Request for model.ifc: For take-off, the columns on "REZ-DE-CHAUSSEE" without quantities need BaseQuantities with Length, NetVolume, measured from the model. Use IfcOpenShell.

First a look at what the model holds.

```python
import ifcopenshell
import ifcopenshell.util.element
import ifcopenshell.util.unit

model = ifcopenshell.open("model.ifc")
print(model.schema)
for unit_type in ("LENGTHUNIT", "AREAUNIT", "VOLUMEUNIT"):
    print(unit_type, ifcopenshell.util.unit.calculate_unit_scale(model, unit_type))
storey = next(s for s in model.by_type("IfcBuildingStorey") if s.Name == "REZ-DE-CHAUSSEE")
columns = [e for e in ifcopenshell.util.element.get_decomposition(storey) if e.is_a("IfcColumn")]
for e in sorted(columns, key=lambda e: e.id()):
    print(e.id(), e.is_a(), e.Name, list(ifcopenshell.util.element.get_psets(e, qtos_only=True)), sep=" | ")
```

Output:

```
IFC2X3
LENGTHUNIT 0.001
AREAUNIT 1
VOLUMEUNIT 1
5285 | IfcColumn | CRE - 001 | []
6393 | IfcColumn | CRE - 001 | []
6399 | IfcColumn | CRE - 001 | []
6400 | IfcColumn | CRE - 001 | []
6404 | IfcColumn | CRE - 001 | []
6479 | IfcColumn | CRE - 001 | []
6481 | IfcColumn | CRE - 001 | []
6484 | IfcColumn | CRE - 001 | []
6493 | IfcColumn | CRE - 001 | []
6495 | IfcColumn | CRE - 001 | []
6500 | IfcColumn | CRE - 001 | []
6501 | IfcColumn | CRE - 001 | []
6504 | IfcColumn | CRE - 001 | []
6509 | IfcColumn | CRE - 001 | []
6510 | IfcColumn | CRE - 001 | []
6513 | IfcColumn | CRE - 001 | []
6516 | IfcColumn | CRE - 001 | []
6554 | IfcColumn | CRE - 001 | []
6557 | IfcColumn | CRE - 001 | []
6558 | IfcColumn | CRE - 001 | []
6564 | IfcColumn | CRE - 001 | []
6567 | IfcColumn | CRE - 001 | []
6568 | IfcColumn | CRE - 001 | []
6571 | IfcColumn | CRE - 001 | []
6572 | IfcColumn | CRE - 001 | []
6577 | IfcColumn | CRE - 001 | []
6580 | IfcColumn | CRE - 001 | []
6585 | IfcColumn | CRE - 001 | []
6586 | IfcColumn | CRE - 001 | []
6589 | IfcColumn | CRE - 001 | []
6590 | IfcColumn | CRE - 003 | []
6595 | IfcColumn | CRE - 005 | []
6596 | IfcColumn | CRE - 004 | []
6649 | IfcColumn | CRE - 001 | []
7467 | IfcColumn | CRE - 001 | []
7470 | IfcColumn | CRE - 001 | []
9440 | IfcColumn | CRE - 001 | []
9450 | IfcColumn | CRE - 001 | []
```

```python
import ifcopenshell
import ifcopenshell.api.pset
import ifcopenshell.geom
import ifcopenshell.util.element
import ifcopenshell.util.shape
import ifcopenshell.util.unit

model = ifcopenshell.open("model.ifc")
unit_scale = ifcopenshell.util.unit.calculate_unit_scale(model)
volume_scale = ifcopenshell.util.unit.calculate_unit_scale(model, "VOLUMEUNIT")
settings = ifcopenshell.geom.settings()

storey = next(s for s in model.by_type("IfcBuildingStorey") if s.Name == "REZ-DE-CHAUSSEE")
columns = [e for e in ifcopenshell.util.element.get_decomposition(storey) if e.is_a("IfcColumn")]

for e in sorted(columns, key=lambda e: e.id()):
    if ifcopenshell.util.element.get_psets(e, qtos_only=True, should_inherit=False):
        continue
    # Geometry comes back in metres, in the element's own axes.
    shape = ifcopenshell.geom.create_shape(settings, e)
    values = {
        "Length": ifcopenshell.util.shape.get_z(shape.geometry) / unit_scale,
        "NetVolume": ifcopenshell.util.shape.get_volume(shape.geometry) / volume_scale,
    }
    qto = ifcopenshell.api.pset.add_qto(model, product=e, name="BaseQuantities")
    ifcopenshell.api.pset.edit_qto(model, qto=qto, properties=values)
    print(e.id(), {k: round(v, 3) for k, v in values.items()})

model.write("model_rev.ifc")
```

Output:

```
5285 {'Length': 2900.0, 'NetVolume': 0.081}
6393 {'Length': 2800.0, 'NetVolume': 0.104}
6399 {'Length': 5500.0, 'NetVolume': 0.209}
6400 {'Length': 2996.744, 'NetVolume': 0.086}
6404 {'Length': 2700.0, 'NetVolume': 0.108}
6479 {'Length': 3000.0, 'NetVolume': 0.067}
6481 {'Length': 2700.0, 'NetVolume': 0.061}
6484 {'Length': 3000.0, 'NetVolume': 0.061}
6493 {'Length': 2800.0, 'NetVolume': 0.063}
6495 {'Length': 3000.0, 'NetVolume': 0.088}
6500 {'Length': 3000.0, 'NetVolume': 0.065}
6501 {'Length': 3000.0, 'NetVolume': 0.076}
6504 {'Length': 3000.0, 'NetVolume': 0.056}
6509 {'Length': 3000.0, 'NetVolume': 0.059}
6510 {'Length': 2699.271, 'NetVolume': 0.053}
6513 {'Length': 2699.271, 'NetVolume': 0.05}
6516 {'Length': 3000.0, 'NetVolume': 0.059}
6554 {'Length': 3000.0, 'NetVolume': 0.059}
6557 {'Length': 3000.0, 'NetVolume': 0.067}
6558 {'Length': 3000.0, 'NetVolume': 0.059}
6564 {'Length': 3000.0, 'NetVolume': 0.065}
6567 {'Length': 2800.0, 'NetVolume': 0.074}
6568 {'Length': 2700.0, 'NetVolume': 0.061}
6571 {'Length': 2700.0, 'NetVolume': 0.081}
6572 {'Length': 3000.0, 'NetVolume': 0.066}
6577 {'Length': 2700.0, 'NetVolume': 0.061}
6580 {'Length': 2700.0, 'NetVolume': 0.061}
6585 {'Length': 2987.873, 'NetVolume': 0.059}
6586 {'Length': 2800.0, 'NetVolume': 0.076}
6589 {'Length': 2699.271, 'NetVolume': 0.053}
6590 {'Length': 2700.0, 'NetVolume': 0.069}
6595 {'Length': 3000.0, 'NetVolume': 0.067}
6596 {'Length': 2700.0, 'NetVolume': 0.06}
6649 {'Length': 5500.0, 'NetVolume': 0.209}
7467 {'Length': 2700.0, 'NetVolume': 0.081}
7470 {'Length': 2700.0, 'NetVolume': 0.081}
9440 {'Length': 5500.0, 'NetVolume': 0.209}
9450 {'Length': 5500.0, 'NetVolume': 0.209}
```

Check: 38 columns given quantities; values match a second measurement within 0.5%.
